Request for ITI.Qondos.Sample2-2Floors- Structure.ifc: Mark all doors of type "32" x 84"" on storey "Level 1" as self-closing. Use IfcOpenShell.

First a look at what the model holds.

```python
import ifcopenshell
import ifcopenshell.util.element

model = ifcopenshell.open("ITI.Qondos.Sample2-2Floors- Structure.ifc")
print(model.schema)
storey = next(s for s in model.by_type("IfcBuildingStorey") if s.Name == "Level 1")
doors = [e for e in ifcopenshell.util.element.get_decomposition(storey) if e.is_a("IfcDoor")]
seen = {}
for e in doors:
    element_type = ifcopenshell.util.element.get_type(e)
    key = (element_type.Name if element_type != e and element_type else None, ifcopenshell.util.element.get_pset(e, "Pset_DoorCommon", "SelfClosing"))
    seen[key] = seen.get(key, 0) + 1
for (name, value), count in sorted(seen.items(), key=str):
    print(count, "x", name, "|", value)
```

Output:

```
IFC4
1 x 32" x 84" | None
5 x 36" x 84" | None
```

```python
import ifcopenshell
import ifcopenshell.api.pset
import ifcopenshell.util.element

model = ifcopenshell.open("ITI.Qondos.Sample2-2Floors- Structure.ifc")

storey = next(s for s in model.by_type("IfcBuildingStorey") if s.Name == "Level 1")
doors = [e for e in ifcopenshell.util.element.get_decomposition(storey) if e.is_a("IfcDoor")]

count = 0
for e in doors:
    element_type = ifcopenshell.util.element.get_type(e)
    if element_type in (None, e) or element_type.Name != '32" x 84"':
        continue
    # add_pset returns the element's existing set when there is one.
    pset = ifcopenshell.api.pset.add_pset(model, product=e, name="Pset_DoorCommon")
    ifcopenshell.api.pset.edit_pset(model, pset=pset, properties={"SelfClosing": True})
    count += 1

print(count, "doors updated")

model.write("ITI.Qondos.Sample2-2Floors- Structure_rev.ifc")
```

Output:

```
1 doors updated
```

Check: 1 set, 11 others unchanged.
